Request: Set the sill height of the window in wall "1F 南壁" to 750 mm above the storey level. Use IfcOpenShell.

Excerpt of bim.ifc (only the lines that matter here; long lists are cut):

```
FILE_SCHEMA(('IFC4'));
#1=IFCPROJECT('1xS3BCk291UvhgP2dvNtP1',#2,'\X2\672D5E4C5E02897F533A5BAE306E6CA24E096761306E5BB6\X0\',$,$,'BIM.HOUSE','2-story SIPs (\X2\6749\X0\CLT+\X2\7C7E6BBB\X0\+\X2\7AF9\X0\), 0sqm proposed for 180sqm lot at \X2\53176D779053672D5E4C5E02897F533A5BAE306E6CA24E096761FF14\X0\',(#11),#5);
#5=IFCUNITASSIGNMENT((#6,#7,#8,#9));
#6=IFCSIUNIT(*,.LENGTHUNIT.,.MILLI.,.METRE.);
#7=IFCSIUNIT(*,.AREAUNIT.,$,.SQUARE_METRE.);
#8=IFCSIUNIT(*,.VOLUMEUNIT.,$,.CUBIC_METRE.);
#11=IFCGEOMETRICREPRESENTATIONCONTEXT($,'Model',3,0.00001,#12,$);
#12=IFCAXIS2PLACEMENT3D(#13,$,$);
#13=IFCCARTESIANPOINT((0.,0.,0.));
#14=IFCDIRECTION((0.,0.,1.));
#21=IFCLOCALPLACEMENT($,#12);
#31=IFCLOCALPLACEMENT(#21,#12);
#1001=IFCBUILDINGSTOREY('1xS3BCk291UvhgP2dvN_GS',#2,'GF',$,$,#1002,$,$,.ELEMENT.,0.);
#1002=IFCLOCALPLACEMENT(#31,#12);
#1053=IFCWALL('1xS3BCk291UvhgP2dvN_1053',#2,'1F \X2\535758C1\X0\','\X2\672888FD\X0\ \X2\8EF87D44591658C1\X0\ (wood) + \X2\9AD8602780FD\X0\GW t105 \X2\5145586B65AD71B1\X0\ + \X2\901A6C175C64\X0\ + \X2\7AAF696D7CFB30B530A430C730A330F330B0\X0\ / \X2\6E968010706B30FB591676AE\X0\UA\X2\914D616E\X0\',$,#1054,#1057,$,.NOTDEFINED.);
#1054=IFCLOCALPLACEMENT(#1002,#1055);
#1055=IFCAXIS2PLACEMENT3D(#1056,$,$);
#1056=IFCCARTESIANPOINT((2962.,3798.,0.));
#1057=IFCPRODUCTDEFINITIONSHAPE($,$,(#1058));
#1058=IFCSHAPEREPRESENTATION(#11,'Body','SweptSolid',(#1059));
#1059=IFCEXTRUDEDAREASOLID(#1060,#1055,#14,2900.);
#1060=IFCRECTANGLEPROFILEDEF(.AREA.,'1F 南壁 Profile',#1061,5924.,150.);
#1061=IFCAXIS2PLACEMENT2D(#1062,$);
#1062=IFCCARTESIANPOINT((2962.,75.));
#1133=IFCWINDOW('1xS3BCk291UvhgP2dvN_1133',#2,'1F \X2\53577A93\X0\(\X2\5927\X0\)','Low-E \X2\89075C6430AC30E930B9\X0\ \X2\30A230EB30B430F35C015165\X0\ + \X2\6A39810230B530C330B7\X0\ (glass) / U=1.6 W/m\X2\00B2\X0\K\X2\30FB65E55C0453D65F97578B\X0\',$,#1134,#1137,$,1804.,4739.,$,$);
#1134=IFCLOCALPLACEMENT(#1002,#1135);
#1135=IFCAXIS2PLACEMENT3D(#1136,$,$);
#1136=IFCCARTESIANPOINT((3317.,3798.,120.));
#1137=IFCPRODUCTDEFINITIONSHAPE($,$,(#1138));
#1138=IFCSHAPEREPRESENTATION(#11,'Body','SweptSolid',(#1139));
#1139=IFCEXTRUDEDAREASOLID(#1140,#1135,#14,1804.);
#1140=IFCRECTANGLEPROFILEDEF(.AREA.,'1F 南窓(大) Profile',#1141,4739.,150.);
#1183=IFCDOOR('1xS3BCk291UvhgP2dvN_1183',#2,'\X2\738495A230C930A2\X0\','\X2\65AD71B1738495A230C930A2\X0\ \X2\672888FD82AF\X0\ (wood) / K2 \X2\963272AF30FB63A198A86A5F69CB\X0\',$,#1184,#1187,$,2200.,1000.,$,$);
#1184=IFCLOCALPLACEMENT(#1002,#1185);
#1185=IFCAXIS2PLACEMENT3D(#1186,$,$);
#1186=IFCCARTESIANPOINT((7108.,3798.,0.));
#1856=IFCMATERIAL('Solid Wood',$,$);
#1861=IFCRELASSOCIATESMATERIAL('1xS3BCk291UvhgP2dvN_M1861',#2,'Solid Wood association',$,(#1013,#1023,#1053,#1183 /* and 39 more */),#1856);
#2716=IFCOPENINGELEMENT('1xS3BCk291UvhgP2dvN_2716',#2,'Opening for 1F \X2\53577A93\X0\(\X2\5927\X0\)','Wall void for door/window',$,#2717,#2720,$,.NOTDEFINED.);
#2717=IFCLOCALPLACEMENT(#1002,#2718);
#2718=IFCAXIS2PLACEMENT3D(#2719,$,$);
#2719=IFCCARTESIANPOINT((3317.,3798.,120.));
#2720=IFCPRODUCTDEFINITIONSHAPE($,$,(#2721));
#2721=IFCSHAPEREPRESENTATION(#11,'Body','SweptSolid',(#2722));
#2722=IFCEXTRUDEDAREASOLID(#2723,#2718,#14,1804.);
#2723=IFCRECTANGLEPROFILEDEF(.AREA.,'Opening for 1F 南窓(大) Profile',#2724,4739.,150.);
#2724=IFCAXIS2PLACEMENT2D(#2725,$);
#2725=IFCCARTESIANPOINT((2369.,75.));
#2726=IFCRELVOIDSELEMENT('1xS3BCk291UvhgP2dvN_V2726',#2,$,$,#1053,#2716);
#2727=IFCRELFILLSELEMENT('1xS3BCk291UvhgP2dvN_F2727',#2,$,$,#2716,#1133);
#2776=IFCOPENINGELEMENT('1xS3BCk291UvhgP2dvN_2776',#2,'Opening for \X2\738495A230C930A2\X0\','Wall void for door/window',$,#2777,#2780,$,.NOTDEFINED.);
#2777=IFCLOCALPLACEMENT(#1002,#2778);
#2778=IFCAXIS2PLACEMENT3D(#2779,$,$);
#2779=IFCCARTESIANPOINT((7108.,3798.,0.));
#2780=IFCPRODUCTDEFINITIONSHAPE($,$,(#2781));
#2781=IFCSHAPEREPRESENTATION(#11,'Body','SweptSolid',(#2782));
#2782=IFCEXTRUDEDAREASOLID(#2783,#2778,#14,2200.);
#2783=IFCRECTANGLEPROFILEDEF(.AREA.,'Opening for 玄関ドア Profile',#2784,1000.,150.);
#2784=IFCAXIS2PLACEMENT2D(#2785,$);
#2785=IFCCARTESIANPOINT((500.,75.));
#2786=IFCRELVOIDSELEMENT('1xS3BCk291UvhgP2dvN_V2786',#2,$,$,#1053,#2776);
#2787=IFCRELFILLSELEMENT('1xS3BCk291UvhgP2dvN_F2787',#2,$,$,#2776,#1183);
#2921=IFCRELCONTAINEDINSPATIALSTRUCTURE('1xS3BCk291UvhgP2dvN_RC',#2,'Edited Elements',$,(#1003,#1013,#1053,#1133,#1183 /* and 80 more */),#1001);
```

```python
import numpy as np
import ifcopenshell
import ifcopenshell.api.geometry
import ifcopenshell.geom
import ifcopenshell.util.element
import ifcopenshell.util.placement
import ifcopenshell.util.shape
import ifcopenshell.util.unit

model = ifcopenshell.open("bim.ifc")
unit_scale = ifcopenshell.util.unit.calculate_unit_scale(model)

window = model.by_guid("1xS3BCk291UvhgP2dvN_1133")
opening = window.FillsVoids[0].RelatingOpeningElement
storey = ifcopenshell.util.element.get_container(window, ifc_class="IfcBuildingStorey")
level = ifcopenshell.util.placement.get_local_placement(storey.ObjectPlacement)[2, 3]

# The opening's origin need not be at the sill, so measure its lowest point.
shape = ifcopenshell.geom.create_shape(ifcopenshell.geom.settings(), opening)
bottom = ifcopenshell.util.shape.get_shape_bottom_elevation(shape, shape.geometry) / unit_scale
dz = level + 0.75 / unit_scale - bottom

shift = np.array([0.0, 0.0, dz])
# The window is not placed relative to its opening, so move both.
for product in (opening, window):
    matrix = ifcopenshell.util.placement.get_local_placement(product.ObjectPlacement)
    matrix[:3, 3] += shift
    ifcopenshell.api.geometry.edit_object_placement(model, product=product, matrix=matrix, is_si=False)

print(f"moved by {dz * unit_scale:+.3f} m")

model.write("bim_updated.ifc")
```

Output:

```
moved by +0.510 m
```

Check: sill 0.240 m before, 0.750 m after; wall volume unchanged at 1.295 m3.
